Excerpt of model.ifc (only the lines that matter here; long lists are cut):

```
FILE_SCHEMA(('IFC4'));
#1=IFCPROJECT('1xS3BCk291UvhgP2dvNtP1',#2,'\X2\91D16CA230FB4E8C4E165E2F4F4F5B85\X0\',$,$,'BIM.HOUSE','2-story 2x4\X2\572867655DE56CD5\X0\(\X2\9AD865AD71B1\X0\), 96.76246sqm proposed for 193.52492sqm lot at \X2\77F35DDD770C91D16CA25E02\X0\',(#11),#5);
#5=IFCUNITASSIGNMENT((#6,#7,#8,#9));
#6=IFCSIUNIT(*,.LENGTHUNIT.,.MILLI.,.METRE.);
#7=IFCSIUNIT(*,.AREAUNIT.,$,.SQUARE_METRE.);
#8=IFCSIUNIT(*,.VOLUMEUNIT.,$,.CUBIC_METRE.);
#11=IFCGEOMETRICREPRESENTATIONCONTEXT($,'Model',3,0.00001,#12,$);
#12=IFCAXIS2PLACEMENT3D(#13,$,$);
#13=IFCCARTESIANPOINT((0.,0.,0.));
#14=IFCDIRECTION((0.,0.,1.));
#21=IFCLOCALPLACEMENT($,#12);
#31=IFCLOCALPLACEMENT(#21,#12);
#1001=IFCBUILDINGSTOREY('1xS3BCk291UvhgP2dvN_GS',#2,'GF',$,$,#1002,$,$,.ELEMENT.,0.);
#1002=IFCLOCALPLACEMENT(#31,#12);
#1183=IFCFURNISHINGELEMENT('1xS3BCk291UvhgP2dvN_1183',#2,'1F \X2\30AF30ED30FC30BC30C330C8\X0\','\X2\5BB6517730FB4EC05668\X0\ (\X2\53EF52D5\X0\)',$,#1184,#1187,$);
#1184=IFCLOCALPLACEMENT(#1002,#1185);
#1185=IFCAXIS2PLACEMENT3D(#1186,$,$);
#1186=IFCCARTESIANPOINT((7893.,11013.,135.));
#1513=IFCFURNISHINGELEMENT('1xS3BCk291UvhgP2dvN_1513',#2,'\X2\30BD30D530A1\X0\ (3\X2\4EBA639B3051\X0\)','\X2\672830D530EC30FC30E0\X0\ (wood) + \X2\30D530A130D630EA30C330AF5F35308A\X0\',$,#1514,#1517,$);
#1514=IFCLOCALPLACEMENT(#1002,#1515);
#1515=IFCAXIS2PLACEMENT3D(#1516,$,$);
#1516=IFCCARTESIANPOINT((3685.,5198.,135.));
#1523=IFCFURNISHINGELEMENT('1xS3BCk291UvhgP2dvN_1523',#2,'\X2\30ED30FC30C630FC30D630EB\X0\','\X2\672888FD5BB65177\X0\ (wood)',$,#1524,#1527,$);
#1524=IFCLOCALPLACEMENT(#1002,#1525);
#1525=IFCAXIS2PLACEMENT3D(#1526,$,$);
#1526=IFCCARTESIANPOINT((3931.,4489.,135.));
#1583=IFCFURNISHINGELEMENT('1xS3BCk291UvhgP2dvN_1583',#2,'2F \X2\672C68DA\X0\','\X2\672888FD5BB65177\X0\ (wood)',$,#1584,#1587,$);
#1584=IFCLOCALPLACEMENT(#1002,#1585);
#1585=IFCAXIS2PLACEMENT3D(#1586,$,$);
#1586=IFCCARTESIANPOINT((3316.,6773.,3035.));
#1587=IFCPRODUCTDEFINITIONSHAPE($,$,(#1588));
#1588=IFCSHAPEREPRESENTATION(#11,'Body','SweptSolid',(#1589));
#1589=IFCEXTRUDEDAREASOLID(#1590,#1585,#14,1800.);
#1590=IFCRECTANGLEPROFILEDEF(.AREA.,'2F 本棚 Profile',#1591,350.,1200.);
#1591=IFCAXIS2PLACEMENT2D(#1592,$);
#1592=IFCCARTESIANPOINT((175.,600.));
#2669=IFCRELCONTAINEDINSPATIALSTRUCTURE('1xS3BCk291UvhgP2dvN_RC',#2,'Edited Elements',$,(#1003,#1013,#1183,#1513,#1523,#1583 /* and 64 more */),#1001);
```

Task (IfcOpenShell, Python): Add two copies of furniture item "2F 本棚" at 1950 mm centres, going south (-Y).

```python
import numpy as np
import ifcopenshell
import ifcopenshell.api.geometry
import ifcopenshell.api.root
import ifcopenshell.util.element
import ifcopenshell.util.placement
import ifcopenshell.util.unit

model = ifcopenshell.open("model.ifc")
unit_scale = ifcopenshell.util.unit.calculate_unit_scale(model)


def reuse_history(source, copy):
    """copy_class also copies each property set's owner history, people and application; keep the originals."""
    for rel in copy.IsDefinedBy:
        if rel.is_a("IfcRelDefinesByProperties") and (history := rel.RelatingPropertyDefinition.OwnerHistory):
            rel.RelatingPropertyDefinition.OwnerHistory = source.OwnerHistory
            ifcopenshell.util.element.remove_deep2(model, history)


source = model.by_guid("1xS3BCk291UvhgP2dvN_1583")
base = ifcopenshell.util.placement.get_local_placement(source.ObjectPlacement)
step = np.array([0.0, -1.0, 0.0]) * 1.95 / unit_scale

for i in range(1, 3):
    copy = ifcopenshell.api.root.copy_class(model, product=source)
    copy.Representation = ifcopenshell.util.element.copy_deep(
        model, source.Representation, exclude=["IfcGeometricRepresentationContext", "IfcRepresentationMap"]
    )
    reuse_history(source, copy)
    matrix = base.copy()
    matrix[:3, 3] += i * step
    print("added at", matrix[:3, 3].round(3) + 0.0)
    ifcopenshell.api.geometry.edit_object_placement(model, product=copy, matrix=matrix, is_si=False)

model.write("model-out.ifc")
```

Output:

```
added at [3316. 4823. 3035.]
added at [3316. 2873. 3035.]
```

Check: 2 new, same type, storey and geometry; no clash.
